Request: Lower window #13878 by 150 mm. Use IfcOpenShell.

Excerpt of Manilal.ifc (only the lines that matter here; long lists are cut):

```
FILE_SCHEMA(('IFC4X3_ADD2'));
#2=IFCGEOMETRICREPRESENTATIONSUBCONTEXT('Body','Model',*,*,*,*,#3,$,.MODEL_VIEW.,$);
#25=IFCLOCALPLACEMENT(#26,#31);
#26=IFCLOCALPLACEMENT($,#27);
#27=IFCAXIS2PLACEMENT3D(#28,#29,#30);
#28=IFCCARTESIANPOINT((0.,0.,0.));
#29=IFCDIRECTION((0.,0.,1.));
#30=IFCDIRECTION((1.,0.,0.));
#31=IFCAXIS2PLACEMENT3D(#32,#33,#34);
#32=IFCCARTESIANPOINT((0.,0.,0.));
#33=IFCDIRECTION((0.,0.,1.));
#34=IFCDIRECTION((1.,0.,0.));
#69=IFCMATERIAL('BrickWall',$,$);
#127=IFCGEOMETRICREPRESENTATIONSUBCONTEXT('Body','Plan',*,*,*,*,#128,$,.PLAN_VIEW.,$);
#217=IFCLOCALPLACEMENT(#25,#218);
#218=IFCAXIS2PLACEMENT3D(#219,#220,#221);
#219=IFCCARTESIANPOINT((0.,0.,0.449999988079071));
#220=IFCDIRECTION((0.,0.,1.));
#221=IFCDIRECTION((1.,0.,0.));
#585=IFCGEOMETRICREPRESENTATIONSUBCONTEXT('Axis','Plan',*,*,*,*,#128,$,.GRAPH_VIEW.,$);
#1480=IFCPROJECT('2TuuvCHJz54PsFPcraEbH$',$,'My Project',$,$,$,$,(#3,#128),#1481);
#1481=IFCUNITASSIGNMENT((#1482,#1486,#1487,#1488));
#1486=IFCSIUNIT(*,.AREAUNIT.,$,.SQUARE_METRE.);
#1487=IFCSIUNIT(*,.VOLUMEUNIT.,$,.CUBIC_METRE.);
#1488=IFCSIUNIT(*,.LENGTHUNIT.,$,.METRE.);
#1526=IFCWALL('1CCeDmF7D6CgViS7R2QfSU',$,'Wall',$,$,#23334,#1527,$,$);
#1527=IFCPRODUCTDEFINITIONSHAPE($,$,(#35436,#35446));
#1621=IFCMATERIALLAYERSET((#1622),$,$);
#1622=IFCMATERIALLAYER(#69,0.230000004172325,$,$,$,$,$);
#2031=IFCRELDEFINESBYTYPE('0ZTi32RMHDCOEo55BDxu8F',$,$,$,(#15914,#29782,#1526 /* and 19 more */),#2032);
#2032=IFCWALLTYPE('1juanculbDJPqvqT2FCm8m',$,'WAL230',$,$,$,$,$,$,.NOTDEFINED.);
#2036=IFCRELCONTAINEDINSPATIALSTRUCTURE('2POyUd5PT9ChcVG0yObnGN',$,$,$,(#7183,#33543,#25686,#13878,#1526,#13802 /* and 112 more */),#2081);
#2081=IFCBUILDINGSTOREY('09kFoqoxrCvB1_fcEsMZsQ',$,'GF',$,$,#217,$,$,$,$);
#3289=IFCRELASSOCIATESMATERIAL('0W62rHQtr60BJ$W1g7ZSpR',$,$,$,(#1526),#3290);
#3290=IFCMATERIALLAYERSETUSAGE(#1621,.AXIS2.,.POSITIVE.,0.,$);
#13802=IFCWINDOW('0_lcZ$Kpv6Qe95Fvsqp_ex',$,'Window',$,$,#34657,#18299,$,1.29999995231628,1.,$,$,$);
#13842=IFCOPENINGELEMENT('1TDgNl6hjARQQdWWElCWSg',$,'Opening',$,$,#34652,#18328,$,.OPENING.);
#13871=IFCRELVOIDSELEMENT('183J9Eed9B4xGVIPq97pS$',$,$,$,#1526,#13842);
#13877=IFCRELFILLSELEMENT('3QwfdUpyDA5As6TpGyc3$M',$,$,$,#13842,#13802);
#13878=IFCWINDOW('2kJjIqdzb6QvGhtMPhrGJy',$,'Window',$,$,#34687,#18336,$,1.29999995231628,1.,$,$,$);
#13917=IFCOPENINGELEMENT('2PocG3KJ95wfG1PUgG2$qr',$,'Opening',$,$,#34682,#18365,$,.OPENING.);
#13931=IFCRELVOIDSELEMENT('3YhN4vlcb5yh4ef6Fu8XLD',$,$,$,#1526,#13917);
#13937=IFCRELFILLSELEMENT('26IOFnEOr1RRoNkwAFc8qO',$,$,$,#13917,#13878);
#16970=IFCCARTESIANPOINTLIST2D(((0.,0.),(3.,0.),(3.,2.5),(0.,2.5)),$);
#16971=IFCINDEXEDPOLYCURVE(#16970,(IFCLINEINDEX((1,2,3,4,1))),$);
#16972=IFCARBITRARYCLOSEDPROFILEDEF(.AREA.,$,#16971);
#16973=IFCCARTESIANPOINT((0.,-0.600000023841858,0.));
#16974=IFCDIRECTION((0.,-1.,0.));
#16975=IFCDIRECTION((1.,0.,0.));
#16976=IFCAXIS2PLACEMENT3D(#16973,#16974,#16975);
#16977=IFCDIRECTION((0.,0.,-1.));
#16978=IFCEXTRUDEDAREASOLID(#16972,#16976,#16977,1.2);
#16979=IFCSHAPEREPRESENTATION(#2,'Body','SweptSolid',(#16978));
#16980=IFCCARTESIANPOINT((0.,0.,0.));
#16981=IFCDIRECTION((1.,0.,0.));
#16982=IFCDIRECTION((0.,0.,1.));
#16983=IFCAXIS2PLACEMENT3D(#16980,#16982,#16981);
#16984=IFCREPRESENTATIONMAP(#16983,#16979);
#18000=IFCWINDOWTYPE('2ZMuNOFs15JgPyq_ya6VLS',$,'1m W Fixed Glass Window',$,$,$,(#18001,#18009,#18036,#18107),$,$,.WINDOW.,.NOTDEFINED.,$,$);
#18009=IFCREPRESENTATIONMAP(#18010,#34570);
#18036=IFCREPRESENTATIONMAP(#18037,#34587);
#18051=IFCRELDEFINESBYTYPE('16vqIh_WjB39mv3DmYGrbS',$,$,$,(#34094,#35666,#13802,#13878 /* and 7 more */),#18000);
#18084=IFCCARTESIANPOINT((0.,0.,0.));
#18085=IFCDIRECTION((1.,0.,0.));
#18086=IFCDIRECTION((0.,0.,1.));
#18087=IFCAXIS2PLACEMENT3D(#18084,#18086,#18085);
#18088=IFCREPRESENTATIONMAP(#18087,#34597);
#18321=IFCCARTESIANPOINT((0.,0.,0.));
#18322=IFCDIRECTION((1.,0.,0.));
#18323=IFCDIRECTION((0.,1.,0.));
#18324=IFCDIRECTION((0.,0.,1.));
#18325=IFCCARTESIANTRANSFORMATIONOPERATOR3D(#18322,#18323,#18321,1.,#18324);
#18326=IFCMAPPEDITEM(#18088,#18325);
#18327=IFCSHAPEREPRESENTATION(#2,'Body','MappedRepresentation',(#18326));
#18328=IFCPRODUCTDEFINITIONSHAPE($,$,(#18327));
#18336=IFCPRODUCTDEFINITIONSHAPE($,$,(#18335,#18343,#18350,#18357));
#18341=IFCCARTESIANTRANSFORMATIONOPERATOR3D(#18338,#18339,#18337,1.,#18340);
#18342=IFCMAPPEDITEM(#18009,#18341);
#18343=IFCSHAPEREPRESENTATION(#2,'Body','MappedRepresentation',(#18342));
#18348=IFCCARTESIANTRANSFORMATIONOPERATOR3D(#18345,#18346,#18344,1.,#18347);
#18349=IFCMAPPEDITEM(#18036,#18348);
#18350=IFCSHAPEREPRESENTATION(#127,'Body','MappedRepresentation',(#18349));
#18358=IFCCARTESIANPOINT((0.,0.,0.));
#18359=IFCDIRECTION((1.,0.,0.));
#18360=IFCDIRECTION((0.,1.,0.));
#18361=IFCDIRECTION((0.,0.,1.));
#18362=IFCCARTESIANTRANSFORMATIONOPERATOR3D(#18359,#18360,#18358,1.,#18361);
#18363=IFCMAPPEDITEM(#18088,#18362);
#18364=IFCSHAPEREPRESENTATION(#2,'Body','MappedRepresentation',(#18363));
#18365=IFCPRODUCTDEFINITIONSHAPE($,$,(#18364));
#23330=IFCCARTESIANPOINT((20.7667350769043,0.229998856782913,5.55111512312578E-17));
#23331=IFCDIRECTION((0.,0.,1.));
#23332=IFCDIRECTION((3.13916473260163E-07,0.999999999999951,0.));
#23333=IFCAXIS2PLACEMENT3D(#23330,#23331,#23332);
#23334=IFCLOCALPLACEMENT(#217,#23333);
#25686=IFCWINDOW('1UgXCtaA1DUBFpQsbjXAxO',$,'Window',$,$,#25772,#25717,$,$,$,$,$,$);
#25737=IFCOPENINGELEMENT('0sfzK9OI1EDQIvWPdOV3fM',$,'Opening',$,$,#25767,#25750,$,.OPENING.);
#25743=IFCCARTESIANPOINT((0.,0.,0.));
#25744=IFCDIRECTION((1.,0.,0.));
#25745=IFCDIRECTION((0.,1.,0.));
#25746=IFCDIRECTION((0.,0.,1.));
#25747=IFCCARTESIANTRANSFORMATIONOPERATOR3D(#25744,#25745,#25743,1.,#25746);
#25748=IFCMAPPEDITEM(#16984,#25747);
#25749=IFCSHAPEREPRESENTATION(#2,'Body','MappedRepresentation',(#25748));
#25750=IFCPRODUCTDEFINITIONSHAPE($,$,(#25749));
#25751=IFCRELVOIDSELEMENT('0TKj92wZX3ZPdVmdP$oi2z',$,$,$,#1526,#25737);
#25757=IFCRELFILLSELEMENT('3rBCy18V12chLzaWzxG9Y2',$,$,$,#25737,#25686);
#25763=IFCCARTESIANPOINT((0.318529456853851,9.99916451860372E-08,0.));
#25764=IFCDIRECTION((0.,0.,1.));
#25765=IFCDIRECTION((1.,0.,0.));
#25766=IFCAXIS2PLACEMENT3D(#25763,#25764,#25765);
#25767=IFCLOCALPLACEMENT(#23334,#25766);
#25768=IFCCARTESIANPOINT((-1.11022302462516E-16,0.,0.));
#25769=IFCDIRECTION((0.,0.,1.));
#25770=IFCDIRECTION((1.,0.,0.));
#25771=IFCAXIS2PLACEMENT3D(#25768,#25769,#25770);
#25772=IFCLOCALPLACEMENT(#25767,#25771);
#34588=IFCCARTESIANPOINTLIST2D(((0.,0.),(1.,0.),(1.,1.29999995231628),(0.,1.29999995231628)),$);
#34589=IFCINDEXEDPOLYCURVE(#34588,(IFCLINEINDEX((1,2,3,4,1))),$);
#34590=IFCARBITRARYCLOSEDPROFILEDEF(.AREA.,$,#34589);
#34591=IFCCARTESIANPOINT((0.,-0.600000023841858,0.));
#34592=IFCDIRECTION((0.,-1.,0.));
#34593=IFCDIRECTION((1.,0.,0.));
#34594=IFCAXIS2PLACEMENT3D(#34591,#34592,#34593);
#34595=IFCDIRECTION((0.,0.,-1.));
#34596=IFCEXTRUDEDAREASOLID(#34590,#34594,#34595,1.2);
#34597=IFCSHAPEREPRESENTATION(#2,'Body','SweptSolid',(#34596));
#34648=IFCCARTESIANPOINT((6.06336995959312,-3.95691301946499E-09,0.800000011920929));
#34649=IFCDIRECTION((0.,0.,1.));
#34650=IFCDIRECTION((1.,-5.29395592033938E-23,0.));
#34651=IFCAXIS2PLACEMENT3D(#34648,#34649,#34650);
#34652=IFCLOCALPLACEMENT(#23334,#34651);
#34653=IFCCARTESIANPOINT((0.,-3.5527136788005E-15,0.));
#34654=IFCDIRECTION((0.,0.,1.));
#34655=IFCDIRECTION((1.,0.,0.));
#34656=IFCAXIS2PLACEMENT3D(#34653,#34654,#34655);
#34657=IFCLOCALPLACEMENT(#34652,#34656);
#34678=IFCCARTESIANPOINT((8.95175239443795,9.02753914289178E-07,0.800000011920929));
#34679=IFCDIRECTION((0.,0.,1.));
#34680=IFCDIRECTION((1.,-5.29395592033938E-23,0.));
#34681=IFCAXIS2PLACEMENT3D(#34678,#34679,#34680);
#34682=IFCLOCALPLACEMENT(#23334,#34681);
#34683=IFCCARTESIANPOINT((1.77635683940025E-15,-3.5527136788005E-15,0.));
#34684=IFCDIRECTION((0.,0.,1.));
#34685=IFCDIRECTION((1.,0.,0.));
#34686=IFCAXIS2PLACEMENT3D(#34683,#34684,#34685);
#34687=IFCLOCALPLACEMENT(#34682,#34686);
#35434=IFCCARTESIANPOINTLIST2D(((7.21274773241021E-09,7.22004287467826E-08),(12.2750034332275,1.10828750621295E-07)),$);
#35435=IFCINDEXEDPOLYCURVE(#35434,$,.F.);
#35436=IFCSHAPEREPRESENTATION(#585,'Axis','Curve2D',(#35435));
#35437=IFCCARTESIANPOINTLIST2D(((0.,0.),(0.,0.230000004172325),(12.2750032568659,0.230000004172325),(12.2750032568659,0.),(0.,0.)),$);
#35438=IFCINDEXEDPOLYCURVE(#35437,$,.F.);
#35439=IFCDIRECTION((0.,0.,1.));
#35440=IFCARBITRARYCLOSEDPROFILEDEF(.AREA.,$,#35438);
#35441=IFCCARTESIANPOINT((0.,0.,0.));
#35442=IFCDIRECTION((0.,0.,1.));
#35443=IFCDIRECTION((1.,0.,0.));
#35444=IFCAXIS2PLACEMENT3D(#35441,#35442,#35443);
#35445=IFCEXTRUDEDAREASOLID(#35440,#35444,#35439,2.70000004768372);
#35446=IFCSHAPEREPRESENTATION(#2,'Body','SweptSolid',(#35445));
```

```python
import numpy as np
import ifcopenshell
import ifcopenshell.api.geometry
import ifcopenshell.util.placement
import ifcopenshell.util.unit

model = ifcopenshell.open("Manilal.ifc")
unit_scale = ifcopenshell.util.unit.calculate_unit_scale(model)

window = model.by_guid("2kJjIqdzb6QvGhtMPhrGJy")
opening = window.FillsVoids[0].RelatingOpeningElement
dz = -0.15

shift = np.array([0.0, 0.0, dz])
# The window is placed relative to its opening, so it follows when the opening moves.
matrix = ifcopenshell.util.placement.get_local_placement(opening.ObjectPlacement)
matrix[:3, 3] += shift
ifcopenshell.api.geometry.edit_object_placement(
    model, product=opening, matrix=matrix, is_si=False, should_transform_children=True
)

print(f"moved by {dz * unit_scale:+.3f} m")

model.write("Manilal_rev.ifc")
```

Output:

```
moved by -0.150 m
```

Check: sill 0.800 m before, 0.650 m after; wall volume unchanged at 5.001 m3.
